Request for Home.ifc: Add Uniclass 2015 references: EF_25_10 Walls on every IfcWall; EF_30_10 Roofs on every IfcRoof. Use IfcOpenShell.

First a look at what the model holds.

```python
import ifcopenshell

model = ifcopenshell.open("Home.ifc")
print(model.schema)
print("classifications:", [c.Name for c in model.by_type("IfcClassification")])
for ifc_class in ("IfcDoor", "IfcRoof", "IfcStair", "IfcWall", "IfcWindow"):
    print(ifc_class, len(model.by_type(ifc_class)))
```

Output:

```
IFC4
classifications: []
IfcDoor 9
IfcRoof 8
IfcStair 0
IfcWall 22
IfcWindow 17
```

```python
import ifcopenshell
import ifcopenshell.api.classification

model = ifcopenshell.open("Home.ifc")

system = ifcopenshell.api.classification.add_classification(model, classification="Uniclass 2015")

codes = {
    "IfcWall": ("EF_25_10", "Walls"),
    "IfcRoof": ("EF_30_10", "Roofs"),
}
for ifc_class, (code, name) in codes.items():
    products = model.by_type(ifc_class)
    ifcopenshell.api.classification.add_reference(
        model, products=products, classification=system, identification=code, name=name
    )
    print(code, len(products))

model.write("Home_rev.ifc")
```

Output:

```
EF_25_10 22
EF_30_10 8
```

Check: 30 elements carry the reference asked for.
